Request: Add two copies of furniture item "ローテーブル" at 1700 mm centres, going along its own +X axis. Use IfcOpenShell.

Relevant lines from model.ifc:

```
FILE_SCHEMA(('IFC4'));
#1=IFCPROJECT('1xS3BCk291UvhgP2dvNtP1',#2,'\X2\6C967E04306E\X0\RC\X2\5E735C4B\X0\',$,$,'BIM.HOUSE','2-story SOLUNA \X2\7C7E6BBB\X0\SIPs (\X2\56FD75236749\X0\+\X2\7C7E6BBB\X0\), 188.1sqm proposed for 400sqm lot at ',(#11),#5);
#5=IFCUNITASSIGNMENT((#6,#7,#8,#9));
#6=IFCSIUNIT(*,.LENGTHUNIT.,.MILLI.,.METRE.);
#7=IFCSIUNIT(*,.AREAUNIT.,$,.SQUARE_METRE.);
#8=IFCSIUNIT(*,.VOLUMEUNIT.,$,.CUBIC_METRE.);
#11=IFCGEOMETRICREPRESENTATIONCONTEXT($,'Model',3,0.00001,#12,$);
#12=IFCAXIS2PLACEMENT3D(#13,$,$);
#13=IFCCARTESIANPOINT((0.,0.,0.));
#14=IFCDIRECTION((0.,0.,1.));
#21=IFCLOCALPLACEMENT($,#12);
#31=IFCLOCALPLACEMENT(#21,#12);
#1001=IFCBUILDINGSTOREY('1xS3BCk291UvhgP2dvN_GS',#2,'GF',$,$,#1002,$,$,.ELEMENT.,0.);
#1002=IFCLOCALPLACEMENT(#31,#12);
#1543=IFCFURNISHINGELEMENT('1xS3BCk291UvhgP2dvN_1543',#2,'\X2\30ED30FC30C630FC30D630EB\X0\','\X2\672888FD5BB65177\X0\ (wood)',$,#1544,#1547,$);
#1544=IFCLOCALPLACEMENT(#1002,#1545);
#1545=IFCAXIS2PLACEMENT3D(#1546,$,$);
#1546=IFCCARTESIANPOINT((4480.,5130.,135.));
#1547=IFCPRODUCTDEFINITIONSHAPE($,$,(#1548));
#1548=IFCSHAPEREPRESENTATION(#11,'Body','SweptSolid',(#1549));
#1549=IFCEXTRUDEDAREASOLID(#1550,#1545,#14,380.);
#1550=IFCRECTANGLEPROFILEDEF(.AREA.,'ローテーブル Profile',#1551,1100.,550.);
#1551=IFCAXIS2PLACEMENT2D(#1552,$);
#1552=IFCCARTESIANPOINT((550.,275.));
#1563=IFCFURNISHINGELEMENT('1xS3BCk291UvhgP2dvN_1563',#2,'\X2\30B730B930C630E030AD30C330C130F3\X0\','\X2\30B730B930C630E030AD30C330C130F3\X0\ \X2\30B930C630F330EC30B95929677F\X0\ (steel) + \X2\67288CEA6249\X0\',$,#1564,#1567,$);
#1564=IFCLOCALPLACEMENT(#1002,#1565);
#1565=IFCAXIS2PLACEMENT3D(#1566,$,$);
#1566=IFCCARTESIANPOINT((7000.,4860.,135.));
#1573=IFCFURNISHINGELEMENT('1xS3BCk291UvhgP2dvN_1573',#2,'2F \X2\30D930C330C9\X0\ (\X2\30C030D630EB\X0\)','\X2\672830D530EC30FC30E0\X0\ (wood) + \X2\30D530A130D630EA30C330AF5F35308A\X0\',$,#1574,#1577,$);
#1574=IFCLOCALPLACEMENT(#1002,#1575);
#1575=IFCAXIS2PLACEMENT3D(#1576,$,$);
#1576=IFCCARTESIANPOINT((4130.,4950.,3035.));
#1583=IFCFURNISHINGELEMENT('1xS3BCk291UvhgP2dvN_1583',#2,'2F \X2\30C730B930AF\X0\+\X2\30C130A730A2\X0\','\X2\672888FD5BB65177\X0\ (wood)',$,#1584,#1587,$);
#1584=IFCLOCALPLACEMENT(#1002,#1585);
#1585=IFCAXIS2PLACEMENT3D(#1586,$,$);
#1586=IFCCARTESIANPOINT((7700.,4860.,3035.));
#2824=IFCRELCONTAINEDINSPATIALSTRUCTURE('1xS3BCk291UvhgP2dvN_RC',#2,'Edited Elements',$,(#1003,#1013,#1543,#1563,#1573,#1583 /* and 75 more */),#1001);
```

```python
import ifcopenshell
import ifcopenshell.api.geometry
import ifcopenshell.api.root
import ifcopenshell.util.element
import ifcopenshell.util.placement

model = ifcopenshell.open("model.ifc")


def reuse_history(source, copy):
    """copy_class also copies each property set's owner history, people and application; keep the originals."""
    for rel in copy.IsDefinedBy:
        if rel.is_a("IfcRelDefinesByProperties") and (history := rel.RelatingPropertyDefinition.OwnerHistory):
            rel.RelatingPropertyDefinition.OwnerHistory = source.OwnerHistory
            ifcopenshell.util.element.remove_deep2(model, history)


source = model.by_guid("1xS3BCk291UvhgP2dvN_1543")
base = ifcopenshell.util.placement.get_local_placement(source.ObjectPlacement)
step = base[:3, 0] * 1700.0

for i in range(1, 3):
    copy = ifcopenshell.api.root.copy_class(model, product=source)
    copy.Representation = ifcopenshell.util.element.copy_deep(
        model, source.Representation, exclude=["IfcGeometricRepresentationContext", "IfcRepresentationMap"]
    )
    reuse_history(source, copy)
    matrix = base.copy()
    matrix[:3, 3] += i * step
    print("added at", matrix[:3, 3].round(3) + 0.0)
    ifcopenshell.api.geometry.edit_object_placement(model, product=copy, matrix=matrix, is_si=False)

model.write("model_updated.ifc")
```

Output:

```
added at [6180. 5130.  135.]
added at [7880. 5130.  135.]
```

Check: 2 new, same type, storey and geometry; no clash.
